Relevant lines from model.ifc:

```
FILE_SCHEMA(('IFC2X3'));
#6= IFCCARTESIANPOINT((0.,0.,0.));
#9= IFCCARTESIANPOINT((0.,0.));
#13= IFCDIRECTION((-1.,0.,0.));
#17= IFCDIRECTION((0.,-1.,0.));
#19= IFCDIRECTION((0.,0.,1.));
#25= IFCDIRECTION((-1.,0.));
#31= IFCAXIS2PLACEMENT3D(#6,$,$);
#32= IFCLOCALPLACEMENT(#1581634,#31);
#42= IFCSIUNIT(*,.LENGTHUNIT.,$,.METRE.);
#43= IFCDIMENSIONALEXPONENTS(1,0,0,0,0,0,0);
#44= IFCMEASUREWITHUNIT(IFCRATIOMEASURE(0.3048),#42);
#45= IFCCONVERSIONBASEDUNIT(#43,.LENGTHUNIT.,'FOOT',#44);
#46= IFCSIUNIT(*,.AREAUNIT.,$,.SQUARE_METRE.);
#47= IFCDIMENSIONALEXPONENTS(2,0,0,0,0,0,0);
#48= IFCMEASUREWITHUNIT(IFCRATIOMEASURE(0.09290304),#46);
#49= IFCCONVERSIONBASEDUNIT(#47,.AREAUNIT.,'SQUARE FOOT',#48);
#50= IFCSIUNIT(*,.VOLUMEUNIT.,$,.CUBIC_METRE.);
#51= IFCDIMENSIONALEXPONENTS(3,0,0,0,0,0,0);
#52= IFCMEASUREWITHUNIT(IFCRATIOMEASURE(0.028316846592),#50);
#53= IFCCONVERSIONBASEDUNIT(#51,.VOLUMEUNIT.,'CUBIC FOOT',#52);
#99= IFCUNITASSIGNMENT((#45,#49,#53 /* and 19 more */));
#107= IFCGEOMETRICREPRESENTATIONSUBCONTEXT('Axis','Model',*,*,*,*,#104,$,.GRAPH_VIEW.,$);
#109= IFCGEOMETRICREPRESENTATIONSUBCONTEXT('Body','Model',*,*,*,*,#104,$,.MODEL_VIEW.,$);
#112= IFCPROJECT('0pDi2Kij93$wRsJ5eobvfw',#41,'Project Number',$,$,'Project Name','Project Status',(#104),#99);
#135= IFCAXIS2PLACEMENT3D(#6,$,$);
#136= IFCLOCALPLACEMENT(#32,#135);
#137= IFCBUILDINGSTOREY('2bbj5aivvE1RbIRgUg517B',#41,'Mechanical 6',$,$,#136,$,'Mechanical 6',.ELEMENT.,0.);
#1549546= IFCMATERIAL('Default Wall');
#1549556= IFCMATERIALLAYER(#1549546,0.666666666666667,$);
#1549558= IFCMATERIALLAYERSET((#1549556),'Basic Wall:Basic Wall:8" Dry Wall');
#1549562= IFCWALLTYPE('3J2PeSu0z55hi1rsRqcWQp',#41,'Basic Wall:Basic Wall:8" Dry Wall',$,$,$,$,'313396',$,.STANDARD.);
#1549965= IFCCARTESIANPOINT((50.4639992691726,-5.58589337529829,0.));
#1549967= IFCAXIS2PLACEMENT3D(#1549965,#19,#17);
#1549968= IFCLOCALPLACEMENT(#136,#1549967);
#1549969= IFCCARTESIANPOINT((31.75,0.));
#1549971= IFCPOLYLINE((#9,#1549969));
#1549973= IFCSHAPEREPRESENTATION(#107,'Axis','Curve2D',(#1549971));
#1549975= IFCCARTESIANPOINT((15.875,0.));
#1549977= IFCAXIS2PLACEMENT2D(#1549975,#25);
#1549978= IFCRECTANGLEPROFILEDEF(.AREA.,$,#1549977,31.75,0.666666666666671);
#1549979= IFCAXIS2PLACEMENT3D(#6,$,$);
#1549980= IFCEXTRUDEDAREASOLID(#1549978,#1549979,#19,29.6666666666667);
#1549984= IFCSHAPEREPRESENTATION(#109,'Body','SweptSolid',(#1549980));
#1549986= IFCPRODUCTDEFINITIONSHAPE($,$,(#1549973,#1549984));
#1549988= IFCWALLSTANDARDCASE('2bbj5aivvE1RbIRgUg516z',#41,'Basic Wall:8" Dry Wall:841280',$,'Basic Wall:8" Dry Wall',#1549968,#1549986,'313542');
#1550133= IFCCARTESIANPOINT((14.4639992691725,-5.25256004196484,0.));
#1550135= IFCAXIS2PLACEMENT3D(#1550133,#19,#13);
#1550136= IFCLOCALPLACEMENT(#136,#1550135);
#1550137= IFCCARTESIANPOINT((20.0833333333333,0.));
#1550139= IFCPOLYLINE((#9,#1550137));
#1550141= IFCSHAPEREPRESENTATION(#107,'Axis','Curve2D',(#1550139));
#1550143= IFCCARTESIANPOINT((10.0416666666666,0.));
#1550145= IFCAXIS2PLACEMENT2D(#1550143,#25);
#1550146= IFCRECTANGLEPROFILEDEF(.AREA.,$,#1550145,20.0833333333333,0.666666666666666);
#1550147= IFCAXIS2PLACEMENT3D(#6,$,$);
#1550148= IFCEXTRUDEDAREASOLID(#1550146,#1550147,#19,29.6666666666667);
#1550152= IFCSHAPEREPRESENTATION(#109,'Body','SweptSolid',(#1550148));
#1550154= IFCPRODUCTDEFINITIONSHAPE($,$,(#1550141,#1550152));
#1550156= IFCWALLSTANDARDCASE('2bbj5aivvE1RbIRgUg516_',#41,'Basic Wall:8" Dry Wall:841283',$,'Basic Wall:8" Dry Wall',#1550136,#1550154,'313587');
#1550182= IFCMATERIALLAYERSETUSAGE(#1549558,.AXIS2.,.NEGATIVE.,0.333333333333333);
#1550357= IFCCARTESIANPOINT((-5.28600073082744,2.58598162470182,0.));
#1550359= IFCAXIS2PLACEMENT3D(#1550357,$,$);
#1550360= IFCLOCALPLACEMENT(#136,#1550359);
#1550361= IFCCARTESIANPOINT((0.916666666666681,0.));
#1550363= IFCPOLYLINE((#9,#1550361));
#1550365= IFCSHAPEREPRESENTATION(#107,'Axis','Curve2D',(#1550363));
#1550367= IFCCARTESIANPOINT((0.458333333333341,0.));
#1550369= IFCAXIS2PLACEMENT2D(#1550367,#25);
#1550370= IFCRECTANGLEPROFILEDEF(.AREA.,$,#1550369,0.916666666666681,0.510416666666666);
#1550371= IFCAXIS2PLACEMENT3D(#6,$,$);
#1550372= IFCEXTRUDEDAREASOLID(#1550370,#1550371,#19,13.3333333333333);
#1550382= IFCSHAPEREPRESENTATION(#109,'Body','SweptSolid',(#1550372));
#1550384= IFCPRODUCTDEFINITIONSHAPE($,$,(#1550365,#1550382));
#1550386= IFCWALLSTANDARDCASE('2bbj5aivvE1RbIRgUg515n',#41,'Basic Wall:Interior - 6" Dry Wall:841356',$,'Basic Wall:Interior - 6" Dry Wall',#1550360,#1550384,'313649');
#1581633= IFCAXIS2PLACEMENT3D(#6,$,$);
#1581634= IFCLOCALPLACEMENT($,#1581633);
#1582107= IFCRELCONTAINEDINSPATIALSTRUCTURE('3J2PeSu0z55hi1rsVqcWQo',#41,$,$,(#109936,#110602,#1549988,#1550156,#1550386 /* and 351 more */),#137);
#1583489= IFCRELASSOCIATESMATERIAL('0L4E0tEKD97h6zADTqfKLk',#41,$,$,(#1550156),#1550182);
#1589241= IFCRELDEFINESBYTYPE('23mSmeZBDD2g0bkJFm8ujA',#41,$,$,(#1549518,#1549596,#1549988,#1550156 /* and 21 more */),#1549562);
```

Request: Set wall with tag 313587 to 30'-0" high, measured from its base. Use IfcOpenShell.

```python
import ifcopenshell
import ifcopenshell.geom
import ifcopenshell.util.representation
import ifcopenshell.util.shape
import ifcopenshell.util.unit

model = ifcopenshell.open("model.ifc")
unit_scale = ifcopenshell.util.unit.calculate_unit_scale(model)
settings = ifcopenshell.geom.settings()


def volume(element):
    """Net volume in cubic metres, openings subtracted."""
    shape = ifcopenshell.geom.create_shape(settings, element)
    return ifcopenshell.util.shape.get_volume(shape.geometry)


wall = model.by_guid("2bbj5aivvE1RbIRgUg516_")
before = volume(wall)

body = ifcopenshell.util.representation.get_representation(wall, "Model", "Body")
solid = body.Items[0]
old_height = solid.Depth
solid.Depth = 360 * 0.0254 / unit_scale
after = volume(wall)

print(f"height {old_height:g} -> {solid.Depth:g}, volume {before:.3f} -> {after:.3f} m3")

model.write("model-out.ifc")
```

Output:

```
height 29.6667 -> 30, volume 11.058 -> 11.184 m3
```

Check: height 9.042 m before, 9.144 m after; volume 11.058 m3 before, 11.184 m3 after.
